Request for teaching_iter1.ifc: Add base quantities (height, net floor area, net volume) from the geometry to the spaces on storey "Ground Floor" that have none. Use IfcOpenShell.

First a look at what the model holds.

```python
import ifcopenshell
import ifcopenshell.util.element
import ifcopenshell.util.unit

model = ifcopenshell.open("teaching_iter1.ifc")
print(model.schema)
for unit_type in ("LENGTHUNIT", "AREAUNIT", "VOLUMEUNIT"):
    print(unit_type, ifcopenshell.util.unit.calculate_unit_scale(model, unit_type))
storey = next(s for s in model.by_type("IfcBuildingStorey") if s.Name == "Ground Floor")
spaces = [e for e in ifcopenshell.util.element.get_decomposition(storey) if e.is_a("IfcSpace")]
for e in sorted(spaces, key=lambda e: e.id()):
    print(e.id(), e.is_a(), e.Name, list(ifcopenshell.util.element.get_psets(e, qtos_only=True)), sep=" | ")
```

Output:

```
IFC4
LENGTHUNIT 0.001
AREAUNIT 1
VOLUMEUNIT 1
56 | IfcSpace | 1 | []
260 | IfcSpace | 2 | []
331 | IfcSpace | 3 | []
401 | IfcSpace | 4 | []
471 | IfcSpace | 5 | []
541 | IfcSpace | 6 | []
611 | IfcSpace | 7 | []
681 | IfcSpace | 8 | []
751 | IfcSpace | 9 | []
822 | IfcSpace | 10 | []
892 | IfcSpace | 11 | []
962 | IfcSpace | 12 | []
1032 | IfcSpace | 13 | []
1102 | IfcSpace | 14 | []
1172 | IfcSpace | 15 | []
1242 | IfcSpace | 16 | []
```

```python
import ifcopenshell
import ifcopenshell.api.pset
import ifcopenshell.geom
import ifcopenshell.util.element
import ifcopenshell.util.shape
import ifcopenshell.util.unit

model = ifcopenshell.open("teaching_iter1.ifc")
unit_scale = ifcopenshell.util.unit.calculate_unit_scale(model)
area_scale = ifcopenshell.util.unit.calculate_unit_scale(model, "AREAUNIT")
volume_scale = ifcopenshell.util.unit.calculate_unit_scale(model, "VOLUMEUNIT")
settings = ifcopenshell.geom.settings()

storey = next(s for s in model.by_type("IfcBuildingStorey") if s.Name == "Ground Floor")
spaces = [e for e in ifcopenshell.util.element.get_decomposition(storey) if e.is_a("IfcSpace")]

for e in sorted(spaces, key=lambda e: e.id()):
    if ifcopenshell.util.element.get_psets(e, qtos_only=True, should_inherit=False):
        continue
    # Geometry comes back in metres, in the element's own axes.
    shape = ifcopenshell.geom.create_shape(settings, e)
    values = {
        "Height": ifcopenshell.util.shape.get_z(shape.geometry) / unit_scale,
        "NetFloorArea": ifcopenshell.util.shape.get_footprint_area(shape.geometry) / area_scale,
        "NetVolume": ifcopenshell.util.shape.get_volume(shape.geometry) / volume_scale,
    }
    qto = ifcopenshell.api.pset.add_qto(model, product=e, name="Qto_SpaceBaseQuantities")
    ifcopenshell.api.pset.edit_qto(model, qto=qto, properties=values)
    print(e.id(), {k: round(v, 3) for k, v in values.items()})

model.write("teaching_iter1_v2.ifc")
```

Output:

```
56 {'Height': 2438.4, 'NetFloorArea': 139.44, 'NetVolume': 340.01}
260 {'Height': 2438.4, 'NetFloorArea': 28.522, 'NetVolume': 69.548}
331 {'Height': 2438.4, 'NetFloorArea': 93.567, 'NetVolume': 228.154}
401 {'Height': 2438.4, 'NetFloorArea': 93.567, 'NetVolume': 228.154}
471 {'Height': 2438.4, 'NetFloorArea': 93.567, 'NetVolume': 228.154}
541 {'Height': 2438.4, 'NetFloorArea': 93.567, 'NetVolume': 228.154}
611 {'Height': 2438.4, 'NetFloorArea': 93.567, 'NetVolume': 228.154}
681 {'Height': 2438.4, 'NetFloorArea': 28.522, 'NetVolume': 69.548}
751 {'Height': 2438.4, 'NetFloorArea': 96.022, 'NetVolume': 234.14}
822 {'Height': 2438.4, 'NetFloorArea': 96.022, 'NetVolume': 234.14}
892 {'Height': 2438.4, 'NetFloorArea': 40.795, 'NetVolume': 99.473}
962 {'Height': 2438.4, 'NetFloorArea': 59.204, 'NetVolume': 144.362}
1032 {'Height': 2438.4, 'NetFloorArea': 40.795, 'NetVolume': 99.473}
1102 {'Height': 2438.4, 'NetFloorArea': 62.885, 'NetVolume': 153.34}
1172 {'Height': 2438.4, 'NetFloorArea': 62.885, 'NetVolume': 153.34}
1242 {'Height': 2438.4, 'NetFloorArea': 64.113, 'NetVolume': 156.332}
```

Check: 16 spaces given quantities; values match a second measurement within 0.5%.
